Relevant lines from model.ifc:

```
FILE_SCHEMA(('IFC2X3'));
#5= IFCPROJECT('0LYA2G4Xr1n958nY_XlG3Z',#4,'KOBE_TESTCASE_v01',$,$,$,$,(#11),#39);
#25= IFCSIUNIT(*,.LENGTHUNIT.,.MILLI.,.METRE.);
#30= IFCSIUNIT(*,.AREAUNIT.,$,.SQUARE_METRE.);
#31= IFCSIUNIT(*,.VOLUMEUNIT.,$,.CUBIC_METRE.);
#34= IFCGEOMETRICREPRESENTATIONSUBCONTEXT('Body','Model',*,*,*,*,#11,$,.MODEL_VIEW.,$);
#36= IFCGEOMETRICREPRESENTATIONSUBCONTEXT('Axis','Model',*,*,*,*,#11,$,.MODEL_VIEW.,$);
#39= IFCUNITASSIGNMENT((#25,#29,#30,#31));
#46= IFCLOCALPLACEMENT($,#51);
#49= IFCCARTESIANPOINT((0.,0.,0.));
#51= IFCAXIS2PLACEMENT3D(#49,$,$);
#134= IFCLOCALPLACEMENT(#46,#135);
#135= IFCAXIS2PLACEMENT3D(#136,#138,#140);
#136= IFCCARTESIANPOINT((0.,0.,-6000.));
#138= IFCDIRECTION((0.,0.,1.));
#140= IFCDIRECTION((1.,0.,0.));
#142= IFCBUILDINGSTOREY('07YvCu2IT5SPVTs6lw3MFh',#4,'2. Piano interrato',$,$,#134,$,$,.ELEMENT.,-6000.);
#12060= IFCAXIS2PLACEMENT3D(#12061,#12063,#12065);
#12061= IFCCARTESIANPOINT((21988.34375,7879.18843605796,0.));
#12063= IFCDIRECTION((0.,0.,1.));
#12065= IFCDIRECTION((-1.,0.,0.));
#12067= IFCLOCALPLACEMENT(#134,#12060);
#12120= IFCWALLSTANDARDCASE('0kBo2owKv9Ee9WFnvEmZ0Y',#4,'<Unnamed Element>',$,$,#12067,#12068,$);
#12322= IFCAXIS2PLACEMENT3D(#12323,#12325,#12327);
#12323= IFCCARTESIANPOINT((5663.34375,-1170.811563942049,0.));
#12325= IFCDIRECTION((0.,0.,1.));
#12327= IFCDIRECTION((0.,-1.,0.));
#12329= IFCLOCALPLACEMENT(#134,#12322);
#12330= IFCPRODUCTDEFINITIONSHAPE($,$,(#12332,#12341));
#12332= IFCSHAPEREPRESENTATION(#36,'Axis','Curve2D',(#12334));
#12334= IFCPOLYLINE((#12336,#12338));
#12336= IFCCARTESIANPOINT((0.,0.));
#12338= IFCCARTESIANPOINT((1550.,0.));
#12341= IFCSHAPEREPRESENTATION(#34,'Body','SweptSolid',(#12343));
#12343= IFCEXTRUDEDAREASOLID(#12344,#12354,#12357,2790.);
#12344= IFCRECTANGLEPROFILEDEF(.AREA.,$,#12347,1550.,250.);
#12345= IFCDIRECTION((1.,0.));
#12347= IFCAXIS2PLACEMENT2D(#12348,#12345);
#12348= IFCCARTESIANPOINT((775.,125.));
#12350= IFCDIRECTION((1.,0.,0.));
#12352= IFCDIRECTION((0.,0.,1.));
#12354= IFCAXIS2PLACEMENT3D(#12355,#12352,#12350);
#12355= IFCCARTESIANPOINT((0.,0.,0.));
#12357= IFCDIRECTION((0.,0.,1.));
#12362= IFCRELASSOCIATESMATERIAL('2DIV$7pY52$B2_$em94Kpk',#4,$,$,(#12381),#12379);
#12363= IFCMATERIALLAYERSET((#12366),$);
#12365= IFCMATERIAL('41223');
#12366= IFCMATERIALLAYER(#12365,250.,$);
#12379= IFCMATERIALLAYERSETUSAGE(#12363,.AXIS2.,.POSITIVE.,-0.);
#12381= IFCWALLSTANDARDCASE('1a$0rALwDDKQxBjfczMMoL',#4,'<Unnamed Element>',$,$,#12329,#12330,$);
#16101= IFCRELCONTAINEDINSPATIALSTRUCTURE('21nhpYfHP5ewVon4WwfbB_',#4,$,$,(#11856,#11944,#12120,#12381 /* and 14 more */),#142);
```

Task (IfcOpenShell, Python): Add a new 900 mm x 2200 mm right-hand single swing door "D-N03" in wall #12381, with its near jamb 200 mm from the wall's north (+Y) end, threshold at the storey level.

```python
import numpy as np
import ifcopenshell
import ifcopenshell.api.feature
import ifcopenshell.api.geometry
import ifcopenshell.api.root
import ifcopenshell.api.spatial
import ifcopenshell.api.type
import ifcopenshell.geom
import ifcopenshell.util.element
import ifcopenshell.util.placement
import ifcopenshell.util.representation
import ifcopenshell.util.shape
import ifcopenshell.util.unit

model = ifcopenshell.open("model.ifc")
unit_scale = ifcopenshell.util.unit.calculate_unit_scale(model)
settings = ifcopenshell.geom.settings()


def volume(element):
    """Net volume in cubic metres, openings subtracted."""
    shape = ifcopenshell.geom.create_shape(settings, element)
    return ifcopenshell.util.shape.get_volume(shape.geometry)


wall = model.by_id(12381)
storey = ifcopenshell.util.element.get_container(wall, ifc_class="IfcBuildingStorey")
context = ifcopenshell.util.representation.get_context(model, "Model", "Body", "MODEL_VIEW")
before = volume(wall)

width, height, from_end, sill = 0.9, 2.2, 0.2, 0.0  # metres

# The wall runs along its own X axis, and the end named is its -X end.
wall_shape = ifcopenshell.geom.create_shape(settings, wall)
x, y, z = ifcopenshell.util.shape.get_vertices(wall_shape.geometry).T
start = x.min() + from_end
face, thickness = float(y.min()), float(y.max() - y.min())
wall_matrix = ifcopenshell.util.placement.get_local_placement(wall.ObjectPlacement)
level = ifcopenshell.util.placement.get_local_placement(storey.ObjectPlacement)[2, 3]


def in_wall(x, y):
    """Placement at x, y metres in the wall's axes, at sill height."""
    matrix = wall_matrix.copy()
    matrix[:, 3] = wall_matrix @ np.array([x / unit_scale, y / unit_scale, 0.0, 1.0])
    matrix[2, 3] = level + sill / unit_scale
    return matrix


# Opening: a box that overshoots both wall faces by 50 mm.
opening = ifcopenshell.api.root.create_entity(model, ifc_class="IfcOpeningElement")
box = ifcopenshell.api.geometry.add_wall_representation(
    model, context=context, length=width, height=height, thickness=thickness + 0.1
)
ifcopenshell.api.geometry.assign_representation(model, product=opening, representation=box)
ifcopenshell.api.geometry.edit_object_placement(model, product=opening, matrix=in_wall(start, face - 0.05), is_si=False)
ifcopenshell.api.feature.add_feature(model, feature=opening, element=wall)

door = ifcopenshell.api.root.create_entity(model, ifc_class="IfcDoor", name="D-N03")
door.OverallWidth, door.OverallHeight = width / unit_scale, height / unit_scale
body = ifcopenshell.api.geometry.add_door_representation(
    model,
    context=context,
    overall_width=door.OverallWidth,
    overall_height=door.OverallHeight,
    operation_type="SINGLE_SWING_RIGHT",
    lining_properties={"LiningDepth": thickness / unit_scale, "ThresholdDepth": thickness / unit_scale},
)
ifcopenshell.api.geometry.assign_representation(model, product=door, representation=body)
ifcopenshell.api.spatial.assign_container(model, products=[door], relating_structure=storey)
fills = ifcopenshell.api.feature.add_filling(model, opening=opening, element=door)
fills.OwnerHistory = door.OwnerHistory  # required in IFC2X3

# IFC2X3 keeps the operation on the door style.
style = ifcopenshell.api.root.create_entity(model, ifc_class="IfcDoorStyle", name="D-N03")
style.OperationType, style.ConstructionType = "SINGLE_SWING_RIGHT", "NOTDEFINED"
style.ParameterTakesPrecedence = style.Sizeable = False
ifcopenshell.api.type.assign_type(model, related_objects=[door], relating_type=style)

# The lining spans the wall, so the door starts at the wall face.
ifcopenshell.api.geometry.edit_object_placement(model, product=door, matrix=in_wall(start, face), is_si=False)

after = volume(wall)

print(f"wall volume {before:.3f} -> {after:.3f} m3")

model.write("model_edited.ifc")
```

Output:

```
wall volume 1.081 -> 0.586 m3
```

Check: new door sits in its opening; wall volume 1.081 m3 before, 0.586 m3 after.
